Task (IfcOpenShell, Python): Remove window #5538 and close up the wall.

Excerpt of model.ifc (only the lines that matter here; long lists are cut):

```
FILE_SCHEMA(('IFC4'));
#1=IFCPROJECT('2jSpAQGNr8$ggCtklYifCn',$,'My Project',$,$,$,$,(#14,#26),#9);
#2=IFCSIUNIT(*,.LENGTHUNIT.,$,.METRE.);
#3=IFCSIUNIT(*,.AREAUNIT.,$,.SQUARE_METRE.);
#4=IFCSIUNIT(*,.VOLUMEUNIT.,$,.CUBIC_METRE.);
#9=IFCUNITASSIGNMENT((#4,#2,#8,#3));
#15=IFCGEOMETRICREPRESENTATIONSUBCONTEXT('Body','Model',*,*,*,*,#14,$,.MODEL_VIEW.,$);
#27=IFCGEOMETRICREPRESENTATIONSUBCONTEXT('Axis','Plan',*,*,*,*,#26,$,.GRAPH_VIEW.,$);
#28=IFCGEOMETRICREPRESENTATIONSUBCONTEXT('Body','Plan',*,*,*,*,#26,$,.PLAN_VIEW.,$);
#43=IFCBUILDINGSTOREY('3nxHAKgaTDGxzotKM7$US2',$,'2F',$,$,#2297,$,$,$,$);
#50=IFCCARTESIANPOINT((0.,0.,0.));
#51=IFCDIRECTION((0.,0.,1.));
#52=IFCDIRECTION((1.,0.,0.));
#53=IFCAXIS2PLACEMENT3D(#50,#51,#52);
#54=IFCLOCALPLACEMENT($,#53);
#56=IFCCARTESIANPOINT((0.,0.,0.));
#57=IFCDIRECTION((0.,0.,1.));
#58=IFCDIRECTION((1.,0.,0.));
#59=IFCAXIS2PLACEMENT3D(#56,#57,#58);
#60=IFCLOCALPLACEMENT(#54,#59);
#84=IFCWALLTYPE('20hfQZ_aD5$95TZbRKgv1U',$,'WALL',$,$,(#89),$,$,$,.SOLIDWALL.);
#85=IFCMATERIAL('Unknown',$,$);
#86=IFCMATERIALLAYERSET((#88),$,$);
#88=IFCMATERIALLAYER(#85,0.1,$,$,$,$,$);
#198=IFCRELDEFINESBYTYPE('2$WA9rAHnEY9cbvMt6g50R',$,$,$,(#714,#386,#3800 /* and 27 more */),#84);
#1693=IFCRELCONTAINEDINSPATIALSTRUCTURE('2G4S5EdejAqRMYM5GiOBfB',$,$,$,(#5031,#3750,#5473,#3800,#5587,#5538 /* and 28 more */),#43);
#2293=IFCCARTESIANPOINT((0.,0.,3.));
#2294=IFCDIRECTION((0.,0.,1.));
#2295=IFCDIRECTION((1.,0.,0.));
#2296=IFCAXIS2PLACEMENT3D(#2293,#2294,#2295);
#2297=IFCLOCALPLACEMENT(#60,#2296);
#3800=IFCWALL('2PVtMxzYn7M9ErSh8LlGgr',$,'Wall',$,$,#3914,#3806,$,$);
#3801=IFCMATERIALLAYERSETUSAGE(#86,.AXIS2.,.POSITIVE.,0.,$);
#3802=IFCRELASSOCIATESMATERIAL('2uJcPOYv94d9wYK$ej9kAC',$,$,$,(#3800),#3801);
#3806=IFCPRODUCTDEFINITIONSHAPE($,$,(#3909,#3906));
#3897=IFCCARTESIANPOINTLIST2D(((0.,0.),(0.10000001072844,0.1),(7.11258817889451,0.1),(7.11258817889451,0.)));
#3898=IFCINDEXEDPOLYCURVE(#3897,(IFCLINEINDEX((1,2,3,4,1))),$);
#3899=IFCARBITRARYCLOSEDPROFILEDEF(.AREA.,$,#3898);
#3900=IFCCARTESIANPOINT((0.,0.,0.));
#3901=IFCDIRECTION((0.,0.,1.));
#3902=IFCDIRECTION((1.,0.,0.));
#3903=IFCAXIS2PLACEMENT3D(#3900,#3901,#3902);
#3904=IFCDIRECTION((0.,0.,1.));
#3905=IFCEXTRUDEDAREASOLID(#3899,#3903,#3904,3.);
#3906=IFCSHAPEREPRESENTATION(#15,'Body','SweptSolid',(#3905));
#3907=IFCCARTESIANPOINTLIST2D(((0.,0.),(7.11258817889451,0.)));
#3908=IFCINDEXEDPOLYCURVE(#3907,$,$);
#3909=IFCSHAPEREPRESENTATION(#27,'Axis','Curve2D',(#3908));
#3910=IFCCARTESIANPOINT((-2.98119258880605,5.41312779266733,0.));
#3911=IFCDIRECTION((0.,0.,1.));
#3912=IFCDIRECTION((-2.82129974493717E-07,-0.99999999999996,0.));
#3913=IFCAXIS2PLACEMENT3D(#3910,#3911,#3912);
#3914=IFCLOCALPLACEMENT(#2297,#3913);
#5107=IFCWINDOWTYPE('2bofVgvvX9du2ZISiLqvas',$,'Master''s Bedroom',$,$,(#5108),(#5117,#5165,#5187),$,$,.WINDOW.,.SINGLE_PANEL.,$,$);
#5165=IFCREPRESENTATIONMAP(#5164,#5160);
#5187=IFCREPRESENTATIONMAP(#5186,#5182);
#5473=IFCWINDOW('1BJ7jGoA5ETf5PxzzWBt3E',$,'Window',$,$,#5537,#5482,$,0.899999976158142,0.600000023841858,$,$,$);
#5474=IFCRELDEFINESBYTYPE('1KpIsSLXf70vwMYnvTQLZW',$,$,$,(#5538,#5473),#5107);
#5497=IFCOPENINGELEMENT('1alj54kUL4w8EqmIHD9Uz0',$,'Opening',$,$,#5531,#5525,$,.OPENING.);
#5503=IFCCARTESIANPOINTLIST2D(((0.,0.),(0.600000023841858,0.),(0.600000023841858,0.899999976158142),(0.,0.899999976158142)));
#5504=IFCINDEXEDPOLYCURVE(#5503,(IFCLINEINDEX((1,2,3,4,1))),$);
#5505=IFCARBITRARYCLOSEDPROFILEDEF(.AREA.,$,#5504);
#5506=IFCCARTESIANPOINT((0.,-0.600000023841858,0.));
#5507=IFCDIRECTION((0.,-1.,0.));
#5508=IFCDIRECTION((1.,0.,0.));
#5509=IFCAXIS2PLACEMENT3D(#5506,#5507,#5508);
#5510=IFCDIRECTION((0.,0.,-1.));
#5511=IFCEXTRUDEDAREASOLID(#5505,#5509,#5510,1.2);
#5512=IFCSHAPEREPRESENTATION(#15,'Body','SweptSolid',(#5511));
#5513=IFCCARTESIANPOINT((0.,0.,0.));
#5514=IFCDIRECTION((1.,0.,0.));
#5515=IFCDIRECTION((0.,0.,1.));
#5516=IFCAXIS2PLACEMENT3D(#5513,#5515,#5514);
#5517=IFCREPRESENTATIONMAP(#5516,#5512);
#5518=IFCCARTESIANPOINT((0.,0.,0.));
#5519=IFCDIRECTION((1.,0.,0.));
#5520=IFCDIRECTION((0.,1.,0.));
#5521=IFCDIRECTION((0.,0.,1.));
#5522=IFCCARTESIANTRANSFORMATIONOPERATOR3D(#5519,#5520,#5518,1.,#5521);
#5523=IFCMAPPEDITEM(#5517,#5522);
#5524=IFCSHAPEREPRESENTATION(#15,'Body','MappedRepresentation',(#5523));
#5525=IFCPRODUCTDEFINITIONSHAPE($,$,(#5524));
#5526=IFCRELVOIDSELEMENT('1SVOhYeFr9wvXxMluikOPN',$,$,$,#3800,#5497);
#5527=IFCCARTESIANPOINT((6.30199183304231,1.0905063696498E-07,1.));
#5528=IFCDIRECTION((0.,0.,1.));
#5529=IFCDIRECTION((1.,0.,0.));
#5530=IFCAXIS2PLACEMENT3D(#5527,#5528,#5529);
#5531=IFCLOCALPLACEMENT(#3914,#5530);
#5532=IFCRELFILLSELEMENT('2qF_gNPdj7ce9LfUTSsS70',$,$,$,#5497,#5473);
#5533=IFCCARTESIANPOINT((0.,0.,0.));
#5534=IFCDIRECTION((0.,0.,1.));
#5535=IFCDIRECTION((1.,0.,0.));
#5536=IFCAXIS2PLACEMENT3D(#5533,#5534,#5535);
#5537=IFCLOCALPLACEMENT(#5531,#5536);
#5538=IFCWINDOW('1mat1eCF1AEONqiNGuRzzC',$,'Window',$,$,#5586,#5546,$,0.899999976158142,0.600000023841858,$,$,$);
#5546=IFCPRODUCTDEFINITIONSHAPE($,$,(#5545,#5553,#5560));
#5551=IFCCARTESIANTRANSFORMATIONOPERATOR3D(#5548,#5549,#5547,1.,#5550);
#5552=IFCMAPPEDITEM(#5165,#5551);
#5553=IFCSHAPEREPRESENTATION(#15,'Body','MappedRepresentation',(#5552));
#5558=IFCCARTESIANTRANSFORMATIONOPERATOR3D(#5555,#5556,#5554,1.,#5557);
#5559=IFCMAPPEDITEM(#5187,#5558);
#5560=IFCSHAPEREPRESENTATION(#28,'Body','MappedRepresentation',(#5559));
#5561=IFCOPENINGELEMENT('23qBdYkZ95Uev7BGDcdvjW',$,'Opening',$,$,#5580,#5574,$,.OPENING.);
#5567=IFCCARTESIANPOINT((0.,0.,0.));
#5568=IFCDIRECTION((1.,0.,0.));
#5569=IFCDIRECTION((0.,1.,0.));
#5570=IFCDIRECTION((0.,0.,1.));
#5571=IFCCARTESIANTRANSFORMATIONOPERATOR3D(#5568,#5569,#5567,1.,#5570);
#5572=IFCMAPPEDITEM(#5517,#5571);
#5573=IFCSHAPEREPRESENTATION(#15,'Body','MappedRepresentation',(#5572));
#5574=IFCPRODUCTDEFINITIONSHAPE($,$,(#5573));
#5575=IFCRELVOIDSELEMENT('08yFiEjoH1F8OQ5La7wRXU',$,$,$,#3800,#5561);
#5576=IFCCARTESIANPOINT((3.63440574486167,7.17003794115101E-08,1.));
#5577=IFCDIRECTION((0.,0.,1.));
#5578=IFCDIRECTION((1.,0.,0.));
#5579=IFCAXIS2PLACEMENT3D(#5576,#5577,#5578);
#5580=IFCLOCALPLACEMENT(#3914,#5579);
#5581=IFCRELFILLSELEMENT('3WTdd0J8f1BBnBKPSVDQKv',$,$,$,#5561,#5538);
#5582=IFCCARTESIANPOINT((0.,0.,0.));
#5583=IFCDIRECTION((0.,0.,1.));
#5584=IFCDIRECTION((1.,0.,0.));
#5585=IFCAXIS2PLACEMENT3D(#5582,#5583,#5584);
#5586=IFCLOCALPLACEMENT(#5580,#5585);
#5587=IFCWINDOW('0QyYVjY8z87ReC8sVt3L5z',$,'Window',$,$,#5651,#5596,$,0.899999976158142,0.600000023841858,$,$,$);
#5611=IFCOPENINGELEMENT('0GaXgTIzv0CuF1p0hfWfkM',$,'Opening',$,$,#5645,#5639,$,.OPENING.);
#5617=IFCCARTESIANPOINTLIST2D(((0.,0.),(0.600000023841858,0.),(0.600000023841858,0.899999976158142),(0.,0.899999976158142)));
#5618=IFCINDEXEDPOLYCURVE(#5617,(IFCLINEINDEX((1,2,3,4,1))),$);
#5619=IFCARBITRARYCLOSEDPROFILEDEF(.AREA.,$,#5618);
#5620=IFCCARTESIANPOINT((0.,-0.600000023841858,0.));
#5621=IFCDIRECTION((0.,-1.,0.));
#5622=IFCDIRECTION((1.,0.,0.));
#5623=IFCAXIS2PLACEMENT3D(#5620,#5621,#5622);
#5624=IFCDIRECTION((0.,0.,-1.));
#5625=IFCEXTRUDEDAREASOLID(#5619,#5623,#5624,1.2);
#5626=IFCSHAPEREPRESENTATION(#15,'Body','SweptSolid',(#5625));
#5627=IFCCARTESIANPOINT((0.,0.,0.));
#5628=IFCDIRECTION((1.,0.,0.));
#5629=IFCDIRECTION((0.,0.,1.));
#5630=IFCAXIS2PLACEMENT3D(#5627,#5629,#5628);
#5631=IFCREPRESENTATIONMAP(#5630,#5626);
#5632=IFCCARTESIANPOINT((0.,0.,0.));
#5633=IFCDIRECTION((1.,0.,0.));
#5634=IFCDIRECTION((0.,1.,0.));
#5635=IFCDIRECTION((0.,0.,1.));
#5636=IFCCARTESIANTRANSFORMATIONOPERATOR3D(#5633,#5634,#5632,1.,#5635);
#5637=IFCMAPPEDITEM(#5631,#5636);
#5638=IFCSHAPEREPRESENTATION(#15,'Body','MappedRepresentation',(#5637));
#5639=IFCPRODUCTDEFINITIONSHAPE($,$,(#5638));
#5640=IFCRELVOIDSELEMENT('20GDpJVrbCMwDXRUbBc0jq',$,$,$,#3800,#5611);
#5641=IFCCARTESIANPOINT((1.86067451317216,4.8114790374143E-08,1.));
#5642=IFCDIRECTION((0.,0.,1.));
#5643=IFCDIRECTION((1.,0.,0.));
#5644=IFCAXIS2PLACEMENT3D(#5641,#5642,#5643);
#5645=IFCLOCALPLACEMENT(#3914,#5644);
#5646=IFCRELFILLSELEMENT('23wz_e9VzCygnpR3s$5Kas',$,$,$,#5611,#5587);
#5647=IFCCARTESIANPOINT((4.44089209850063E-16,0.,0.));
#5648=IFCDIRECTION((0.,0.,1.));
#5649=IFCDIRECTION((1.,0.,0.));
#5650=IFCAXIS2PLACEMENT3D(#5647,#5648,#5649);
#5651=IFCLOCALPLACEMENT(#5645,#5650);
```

```python
import ifcopenshell
import ifcopenshell.api.feature
import ifcopenshell.api.root
import ifcopenshell.geom
import ifcopenshell.util.shape

model = ifcopenshell.open("model.ifc")
settings = ifcopenshell.geom.settings()


def volume(element):
    """Net volume in cubic metres, openings subtracted."""
    shape = ifcopenshell.geom.create_shape(settings, element)
    return ifcopenshell.util.shape.get_volume(shape.geometry)


window = model.by_guid("1mat1eCF1AEONqiNGuRzzC")
opening = window.FillsVoids[0].RelatingOpeningElement
wall = opening.VoidsElements[0].RelatingBuildingElement
before = volume(wall)

ifcopenshell.api.root.remove_product(model, product=window)
ifcopenshell.api.feature.remove_feature(model, feature=opening)

after = volume(wall)

print(f"wall volume {before:.3f} -> {after:.3f} m3")

model.write("model_updated.ifc")
```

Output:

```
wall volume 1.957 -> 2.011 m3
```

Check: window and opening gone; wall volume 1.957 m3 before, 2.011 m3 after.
